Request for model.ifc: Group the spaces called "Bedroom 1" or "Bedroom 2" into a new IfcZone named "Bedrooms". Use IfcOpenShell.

First a look at what the model holds.

```python
import ifcopenshell

model = ifcopenshell.open("model.ifc")
print(model.schema)
seen = {}
for space in model.by_type("IfcSpace"):
    seen[space.LongName] = seen.get(space.LongName, 0) + 1
for name, count in sorted(seen.items(), key=str):
    print(count, "x", name)
print("zones:", [z.Name for z in model.by_type("IfcZone")][:20])
```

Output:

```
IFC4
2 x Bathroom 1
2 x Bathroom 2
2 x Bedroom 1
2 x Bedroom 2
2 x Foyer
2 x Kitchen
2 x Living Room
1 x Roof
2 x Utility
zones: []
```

```python
import ifcopenshell
import ifcopenshell.api.group
import ifcopenshell.api.root

model = ifcopenshell.open("model.ifc")

names = {"Bedroom 1", "Bedroom 2"}
spaces = [s for s in model.by_type("IfcSpace") if s.LongName in names]

zone = ifcopenshell.api.root.create_entity(model, ifc_class="IfcZone", name="Bedrooms")
ifcopenshell.api.group.assign_group(model, products=spaces, group=zone)
print(len(spaces), "spaces in", zone.Name)

model.write("model_edited.ifc")
```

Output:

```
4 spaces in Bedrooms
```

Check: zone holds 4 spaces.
